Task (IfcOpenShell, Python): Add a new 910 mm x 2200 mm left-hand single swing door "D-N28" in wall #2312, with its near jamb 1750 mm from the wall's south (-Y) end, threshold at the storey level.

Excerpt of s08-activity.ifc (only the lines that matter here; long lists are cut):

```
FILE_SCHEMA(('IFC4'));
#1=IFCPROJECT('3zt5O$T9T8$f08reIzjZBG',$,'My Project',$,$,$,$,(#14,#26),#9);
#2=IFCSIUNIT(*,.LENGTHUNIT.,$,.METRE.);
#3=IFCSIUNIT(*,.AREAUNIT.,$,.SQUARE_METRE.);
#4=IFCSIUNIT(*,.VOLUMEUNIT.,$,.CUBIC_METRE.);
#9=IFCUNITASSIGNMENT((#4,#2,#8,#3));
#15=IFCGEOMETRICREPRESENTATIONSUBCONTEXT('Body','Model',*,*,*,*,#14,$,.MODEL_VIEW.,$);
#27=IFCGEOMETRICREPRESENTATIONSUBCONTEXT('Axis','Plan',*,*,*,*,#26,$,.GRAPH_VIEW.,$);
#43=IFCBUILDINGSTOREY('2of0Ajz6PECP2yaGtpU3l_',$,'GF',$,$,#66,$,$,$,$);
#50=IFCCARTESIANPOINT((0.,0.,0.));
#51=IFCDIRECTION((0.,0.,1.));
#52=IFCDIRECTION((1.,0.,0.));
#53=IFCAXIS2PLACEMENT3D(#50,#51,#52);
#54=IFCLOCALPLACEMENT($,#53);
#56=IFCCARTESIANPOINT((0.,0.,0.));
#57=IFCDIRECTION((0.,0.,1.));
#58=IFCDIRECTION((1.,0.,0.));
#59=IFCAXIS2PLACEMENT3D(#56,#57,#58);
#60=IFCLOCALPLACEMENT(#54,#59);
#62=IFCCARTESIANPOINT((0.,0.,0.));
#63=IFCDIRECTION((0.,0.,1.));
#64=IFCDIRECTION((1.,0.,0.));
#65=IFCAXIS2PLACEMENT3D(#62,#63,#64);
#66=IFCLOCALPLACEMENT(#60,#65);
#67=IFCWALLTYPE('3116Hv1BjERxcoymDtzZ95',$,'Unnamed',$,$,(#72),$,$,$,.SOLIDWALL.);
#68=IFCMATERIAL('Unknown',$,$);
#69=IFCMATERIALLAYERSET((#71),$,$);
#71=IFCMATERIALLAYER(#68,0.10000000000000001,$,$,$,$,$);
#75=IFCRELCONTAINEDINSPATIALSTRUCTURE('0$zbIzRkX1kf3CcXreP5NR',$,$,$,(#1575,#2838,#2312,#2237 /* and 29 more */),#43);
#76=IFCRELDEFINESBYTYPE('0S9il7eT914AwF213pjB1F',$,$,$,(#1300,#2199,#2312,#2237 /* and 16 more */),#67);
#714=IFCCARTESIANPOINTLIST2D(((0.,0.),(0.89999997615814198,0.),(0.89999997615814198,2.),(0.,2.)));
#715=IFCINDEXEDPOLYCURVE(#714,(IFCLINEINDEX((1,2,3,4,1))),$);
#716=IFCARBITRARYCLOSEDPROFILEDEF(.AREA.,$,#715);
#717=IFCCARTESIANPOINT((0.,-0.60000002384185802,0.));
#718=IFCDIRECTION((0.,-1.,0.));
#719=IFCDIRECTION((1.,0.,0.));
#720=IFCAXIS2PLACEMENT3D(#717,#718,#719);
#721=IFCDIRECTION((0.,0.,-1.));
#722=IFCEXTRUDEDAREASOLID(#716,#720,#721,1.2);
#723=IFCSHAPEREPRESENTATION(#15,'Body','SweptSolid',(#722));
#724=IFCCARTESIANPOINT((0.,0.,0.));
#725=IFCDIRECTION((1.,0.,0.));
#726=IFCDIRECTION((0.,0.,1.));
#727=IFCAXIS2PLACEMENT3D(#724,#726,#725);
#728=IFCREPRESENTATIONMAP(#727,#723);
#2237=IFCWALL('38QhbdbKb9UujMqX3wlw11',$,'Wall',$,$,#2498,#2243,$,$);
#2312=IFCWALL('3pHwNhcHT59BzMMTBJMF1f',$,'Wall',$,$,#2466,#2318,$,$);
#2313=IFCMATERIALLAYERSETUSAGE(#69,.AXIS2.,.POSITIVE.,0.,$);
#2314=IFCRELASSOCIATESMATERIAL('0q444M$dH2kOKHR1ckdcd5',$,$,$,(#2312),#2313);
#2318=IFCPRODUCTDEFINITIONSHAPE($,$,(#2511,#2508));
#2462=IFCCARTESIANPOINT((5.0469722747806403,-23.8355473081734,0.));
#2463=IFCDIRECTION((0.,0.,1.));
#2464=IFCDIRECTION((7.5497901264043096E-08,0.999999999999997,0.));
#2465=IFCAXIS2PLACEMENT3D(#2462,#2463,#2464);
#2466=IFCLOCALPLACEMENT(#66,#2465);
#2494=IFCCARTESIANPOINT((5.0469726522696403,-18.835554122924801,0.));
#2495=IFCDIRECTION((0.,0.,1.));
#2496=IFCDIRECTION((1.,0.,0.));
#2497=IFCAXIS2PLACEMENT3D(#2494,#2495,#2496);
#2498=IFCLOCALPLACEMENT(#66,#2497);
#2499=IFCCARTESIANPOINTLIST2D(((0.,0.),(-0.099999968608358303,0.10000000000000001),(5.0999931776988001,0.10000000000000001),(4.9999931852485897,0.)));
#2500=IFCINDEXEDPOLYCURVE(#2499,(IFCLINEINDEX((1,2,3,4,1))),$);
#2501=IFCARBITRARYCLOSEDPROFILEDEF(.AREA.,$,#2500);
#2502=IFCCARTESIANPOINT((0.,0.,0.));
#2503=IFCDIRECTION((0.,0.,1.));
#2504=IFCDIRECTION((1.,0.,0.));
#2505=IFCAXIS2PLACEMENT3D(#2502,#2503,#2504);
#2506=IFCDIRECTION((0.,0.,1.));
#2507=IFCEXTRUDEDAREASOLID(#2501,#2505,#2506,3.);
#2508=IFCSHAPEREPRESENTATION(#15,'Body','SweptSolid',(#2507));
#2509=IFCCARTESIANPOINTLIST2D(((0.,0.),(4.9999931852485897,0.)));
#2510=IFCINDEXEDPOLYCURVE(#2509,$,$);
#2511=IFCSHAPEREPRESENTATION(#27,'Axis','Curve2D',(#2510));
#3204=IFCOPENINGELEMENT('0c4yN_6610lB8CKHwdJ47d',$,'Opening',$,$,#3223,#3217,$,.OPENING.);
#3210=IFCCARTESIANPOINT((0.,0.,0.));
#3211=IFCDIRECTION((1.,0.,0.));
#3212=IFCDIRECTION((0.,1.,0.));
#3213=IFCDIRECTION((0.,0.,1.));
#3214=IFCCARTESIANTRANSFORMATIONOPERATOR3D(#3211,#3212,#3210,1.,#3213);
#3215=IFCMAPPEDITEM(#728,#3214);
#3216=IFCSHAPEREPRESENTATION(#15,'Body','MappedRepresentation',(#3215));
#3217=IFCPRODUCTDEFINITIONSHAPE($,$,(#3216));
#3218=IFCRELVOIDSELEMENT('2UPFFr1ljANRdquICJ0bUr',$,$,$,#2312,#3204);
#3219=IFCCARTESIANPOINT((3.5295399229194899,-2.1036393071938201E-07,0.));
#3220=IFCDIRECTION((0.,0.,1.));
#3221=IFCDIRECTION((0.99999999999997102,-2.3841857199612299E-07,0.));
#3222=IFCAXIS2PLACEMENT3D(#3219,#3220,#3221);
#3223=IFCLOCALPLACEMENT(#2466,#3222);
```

```python
import numpy as np
import ifcopenshell
import ifcopenshell.api.feature
import ifcopenshell.api.geometry
import ifcopenshell.api.root
import ifcopenshell.api.spatial
import ifcopenshell.geom
import ifcopenshell.util.element
import ifcopenshell.util.placement
import ifcopenshell.util.representation
import ifcopenshell.util.shape
import ifcopenshell.util.unit

model = ifcopenshell.open("s08-activity.ifc")
unit_scale = ifcopenshell.util.unit.calculate_unit_scale(model)
settings = ifcopenshell.geom.settings()


def volume(element):
    """Net volume in cubic metres, openings subtracted."""
    shape = ifcopenshell.geom.create_shape(settings, element)
    return ifcopenshell.util.shape.get_volume(shape.geometry)


wall = model.by_guid("3pHwNhcHT59BzMMTBJMF1f")
storey = ifcopenshell.util.element.get_container(wall, ifc_class="IfcBuildingStorey")
context = ifcopenshell.util.representation.get_context(model, "Model", "Body", "MODEL_VIEW")
before = volume(wall)

width, height, from_end, sill = 0.91, 2.2, 1.75, 0.0  # metres

# The wall runs along its own X axis, and the end named is its -X end.
wall_shape = ifcopenshell.geom.create_shape(settings, wall)
x, y, z = ifcopenshell.util.shape.get_vertices(wall_shape.geometry).T
start = x.min() + from_end
face, thickness = float(y.min()), float(y.max() - y.min())
wall_matrix = ifcopenshell.util.placement.get_local_placement(wall.ObjectPlacement)
level = ifcopenshell.util.placement.get_local_placement(storey.ObjectPlacement)[2, 3]


def in_wall(x, y):
    """Placement at x, y metres in the wall's axes, at sill height."""
    matrix = wall_matrix.copy()
    matrix[:, 3] = wall_matrix @ np.array([x / unit_scale, y / unit_scale, 0.0, 1.0])
    matrix[2, 3] = level + sill / unit_scale
    return matrix


# Opening: a box that overshoots both wall faces by 50 mm.
opening = ifcopenshell.api.root.create_entity(model, ifc_class="IfcOpeningElement", predefined_type="OPENING")
box = ifcopenshell.api.geometry.add_wall_representation(
    model, context=context, length=width, height=height, thickness=thickness + 0.1
)
ifcopenshell.api.geometry.assign_representation(model, product=opening, representation=box)
ifcopenshell.api.geometry.edit_object_placement(model, product=opening, matrix=in_wall(start, face - 0.05), is_si=False)
ifcopenshell.api.feature.add_feature(model, feature=opening, element=wall)

door = ifcopenshell.api.root.create_entity(model, ifc_class="IfcDoor", name="D-N28", predefined_type="DOOR")
door.OverallWidth, door.OverallHeight = width / unit_scale, height / unit_scale
door.OperationType = "SINGLE_SWING_LEFT"
body = ifcopenshell.api.geometry.add_door_representation(
    model,
    context=context,
    overall_width=door.OverallWidth,
    overall_height=door.OverallHeight,
    operation_type="SINGLE_SWING_LEFT",
    lining_properties={"LiningDepth": thickness / unit_scale, "ThresholdDepth": thickness / unit_scale},
)
ifcopenshell.api.geometry.assign_representation(model, product=door, representation=body)
ifcopenshell.api.spatial.assign_container(model, products=[door], relating_structure=storey)
ifcopenshell.api.feature.add_filling(model, opening=opening, element=door)

# The lining spans the wall, so the door starts at the wall face.
ifcopenshell.api.geometry.edit_object_placement(model, product=door, matrix=in_wall(start, face), is_si=False)

after = volume(wall)

print(f"wall volume {before:.3f} -> {after:.3f} m3")

model.write("s08-activity_updated.ifc")
```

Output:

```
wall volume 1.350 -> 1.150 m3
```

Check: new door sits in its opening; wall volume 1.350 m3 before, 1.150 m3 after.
